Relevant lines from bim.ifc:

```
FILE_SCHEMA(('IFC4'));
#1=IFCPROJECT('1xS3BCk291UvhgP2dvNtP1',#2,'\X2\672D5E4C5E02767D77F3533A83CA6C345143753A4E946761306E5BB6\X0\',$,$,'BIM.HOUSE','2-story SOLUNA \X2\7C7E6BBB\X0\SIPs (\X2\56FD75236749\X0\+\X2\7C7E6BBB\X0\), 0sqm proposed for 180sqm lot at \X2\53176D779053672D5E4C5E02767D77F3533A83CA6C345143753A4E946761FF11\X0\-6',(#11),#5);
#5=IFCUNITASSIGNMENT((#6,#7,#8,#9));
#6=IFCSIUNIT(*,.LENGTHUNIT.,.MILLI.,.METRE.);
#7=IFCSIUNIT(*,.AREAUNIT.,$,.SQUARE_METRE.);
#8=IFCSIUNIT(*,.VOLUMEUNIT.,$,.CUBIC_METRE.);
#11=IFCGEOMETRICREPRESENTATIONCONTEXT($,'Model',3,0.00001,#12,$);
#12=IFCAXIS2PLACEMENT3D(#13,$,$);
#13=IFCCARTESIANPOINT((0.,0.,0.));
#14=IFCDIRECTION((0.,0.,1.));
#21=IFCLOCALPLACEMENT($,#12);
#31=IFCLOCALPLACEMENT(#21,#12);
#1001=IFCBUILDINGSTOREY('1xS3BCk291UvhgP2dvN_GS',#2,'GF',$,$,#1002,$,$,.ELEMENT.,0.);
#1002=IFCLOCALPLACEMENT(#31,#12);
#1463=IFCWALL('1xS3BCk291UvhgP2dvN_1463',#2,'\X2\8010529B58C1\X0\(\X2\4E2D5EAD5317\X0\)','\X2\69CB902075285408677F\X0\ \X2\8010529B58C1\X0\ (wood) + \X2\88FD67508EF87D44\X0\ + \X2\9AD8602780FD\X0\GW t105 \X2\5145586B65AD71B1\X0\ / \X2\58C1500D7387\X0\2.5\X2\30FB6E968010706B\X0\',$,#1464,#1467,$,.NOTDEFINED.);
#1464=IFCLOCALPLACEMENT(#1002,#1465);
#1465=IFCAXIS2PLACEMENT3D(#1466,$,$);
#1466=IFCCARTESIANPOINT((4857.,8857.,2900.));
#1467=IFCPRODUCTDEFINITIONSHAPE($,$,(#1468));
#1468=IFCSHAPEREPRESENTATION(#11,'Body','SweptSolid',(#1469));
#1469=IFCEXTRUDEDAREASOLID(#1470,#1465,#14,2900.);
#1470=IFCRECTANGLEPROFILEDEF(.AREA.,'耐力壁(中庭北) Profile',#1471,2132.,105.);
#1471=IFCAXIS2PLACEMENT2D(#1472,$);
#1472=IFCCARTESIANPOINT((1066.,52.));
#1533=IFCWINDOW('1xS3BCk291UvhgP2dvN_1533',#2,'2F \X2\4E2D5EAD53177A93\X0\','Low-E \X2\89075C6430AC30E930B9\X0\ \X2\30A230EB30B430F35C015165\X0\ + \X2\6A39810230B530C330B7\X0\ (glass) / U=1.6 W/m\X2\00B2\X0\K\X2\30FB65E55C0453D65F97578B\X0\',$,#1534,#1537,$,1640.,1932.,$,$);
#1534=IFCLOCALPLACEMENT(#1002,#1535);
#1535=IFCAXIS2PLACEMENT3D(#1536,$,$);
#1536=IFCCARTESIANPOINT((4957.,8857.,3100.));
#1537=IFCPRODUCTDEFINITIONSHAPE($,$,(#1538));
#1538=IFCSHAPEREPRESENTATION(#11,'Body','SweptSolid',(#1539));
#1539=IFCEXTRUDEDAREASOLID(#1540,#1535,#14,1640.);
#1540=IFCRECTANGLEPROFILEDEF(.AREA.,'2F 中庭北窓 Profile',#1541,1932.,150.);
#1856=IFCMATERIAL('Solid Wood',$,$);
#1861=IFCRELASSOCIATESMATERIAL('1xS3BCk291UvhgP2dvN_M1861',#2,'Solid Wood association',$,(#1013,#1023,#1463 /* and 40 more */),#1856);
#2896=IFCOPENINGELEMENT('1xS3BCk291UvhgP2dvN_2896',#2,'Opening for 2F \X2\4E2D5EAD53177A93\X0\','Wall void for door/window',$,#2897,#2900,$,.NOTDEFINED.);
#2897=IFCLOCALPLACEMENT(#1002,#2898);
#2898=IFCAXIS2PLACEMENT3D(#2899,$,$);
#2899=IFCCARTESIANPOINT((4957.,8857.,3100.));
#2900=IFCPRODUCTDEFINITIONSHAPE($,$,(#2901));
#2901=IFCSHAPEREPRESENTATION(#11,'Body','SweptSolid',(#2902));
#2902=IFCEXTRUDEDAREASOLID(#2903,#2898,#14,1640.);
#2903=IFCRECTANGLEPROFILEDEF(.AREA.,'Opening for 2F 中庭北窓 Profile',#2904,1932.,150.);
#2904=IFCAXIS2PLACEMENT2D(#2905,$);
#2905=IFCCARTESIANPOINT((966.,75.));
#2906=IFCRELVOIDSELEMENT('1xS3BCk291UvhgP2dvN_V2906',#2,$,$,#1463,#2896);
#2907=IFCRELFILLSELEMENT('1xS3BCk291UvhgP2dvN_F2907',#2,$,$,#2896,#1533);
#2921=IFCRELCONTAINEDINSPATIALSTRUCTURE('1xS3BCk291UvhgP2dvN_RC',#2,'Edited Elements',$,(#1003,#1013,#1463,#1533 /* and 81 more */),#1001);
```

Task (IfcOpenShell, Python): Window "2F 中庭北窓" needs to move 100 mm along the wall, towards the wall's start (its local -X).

```python
import ifcopenshell
import ifcopenshell.api.geometry
import ifcopenshell.util.placement

model = ifcopenshell.open("bim.ifc")

window = model.by_guid("1xS3BCk291UvhgP2dvN_1533")
opening = window.FillsVoids[0].RelatingOpeningElement
wall = opening.VoidsElements[0].RelatingBuildingElement

wall_matrix = ifcopenshell.util.placement.get_local_placement(wall.ObjectPlacement)
shift = wall_matrix[:3, 0] * -100.0
before = ifcopenshell.util.placement.get_local_placement(window.ObjectPlacement)[:3, 3].copy()

# The window is not placed relative to its opening, so move both.
for product in (opening, window):
    matrix = ifcopenshell.util.placement.get_local_placement(product.ObjectPlacement)
    matrix[:3, 3] += shift
    ifcopenshell.api.geometry.edit_object_placement(model, product=product, matrix=matrix, is_si=False)

after = ifcopenshell.util.placement.get_local_placement(window.ObjectPlacement)[:3, 3]
print("window moved by", (after - before).round(3) + 0.0)

model.write("bim_edited.ifc")
```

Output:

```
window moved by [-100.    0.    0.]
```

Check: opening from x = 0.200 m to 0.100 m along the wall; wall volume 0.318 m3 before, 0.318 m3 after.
